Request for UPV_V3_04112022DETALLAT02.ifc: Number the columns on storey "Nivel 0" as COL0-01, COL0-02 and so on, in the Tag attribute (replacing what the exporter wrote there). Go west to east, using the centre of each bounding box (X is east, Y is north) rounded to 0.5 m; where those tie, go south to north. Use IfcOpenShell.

First a look at what the model holds.

```python
import ifcopenshell
import ifcopenshell.util.element
import ifcopenshell.util.placement

model = ifcopenshell.open("UPV_V3_04112022DETALLAT02.ifc")
print(model.schema)
storey = next(s for s in model.by_type("IfcBuildingStorey") if s.Name == "Nivel 0")
columns = [e for e in ifcopenshell.util.element.get_decomposition(storey) if e.is_a("IfcColumn")]
for e in sorted(columns, key=lambda e: e.id()):
    origin = ifcopenshell.util.placement.get_local_placement(e.ObjectPlacement)[:3, 3]
    print(e.id(), e.Tag, e.Name, origin.round(2) + 0.0, sep=" | ")
```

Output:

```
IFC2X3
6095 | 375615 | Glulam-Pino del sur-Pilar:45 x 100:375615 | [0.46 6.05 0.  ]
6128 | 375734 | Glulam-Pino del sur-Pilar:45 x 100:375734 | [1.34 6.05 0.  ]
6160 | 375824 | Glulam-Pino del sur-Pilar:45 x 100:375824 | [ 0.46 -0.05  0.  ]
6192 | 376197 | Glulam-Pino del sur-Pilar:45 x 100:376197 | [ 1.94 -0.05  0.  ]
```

```python
import ifcopenshell
import ifcopenshell.geom
import ifcopenshell.util.element
import ifcopenshell.util.shape

model = ifcopenshell.open("UPV_V3_04112022DETALLAT02.ifc")
settings = ifcopenshell.geom.settings()
settings.set("use-world-coords", True)


def centre(element):
    shape = ifcopenshell.geom.create_shape(settings, element)
    return ifcopenshell.util.shape.get_bbox_centroid(shape.geometry)


storey = next(s for s in model.by_type("IfcBuildingStorey") if s.Name == "Nivel 0")
columns = [e for e in ifcopenshell.util.element.get_decomposition(storey) if e.is_a("IfcColumn")]

# Insertion points can sit at a corner or the storey origin, so sort by the geometry (in metres).
centres = {e: centre(e) for e in columns}
columns.sort(key=lambda e: (round(centres[e][0] / 0.5), centres[e][1]))

for i, e in enumerate(columns, start=1):
    number = f"COL0-{i:02d}"
    e.Tag = number
    print(e.id(), number)

model.write("UPV_V3_04112022DETALLAT02_updated.ifc")
```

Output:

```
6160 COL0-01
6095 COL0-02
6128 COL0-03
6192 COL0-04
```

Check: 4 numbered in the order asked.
